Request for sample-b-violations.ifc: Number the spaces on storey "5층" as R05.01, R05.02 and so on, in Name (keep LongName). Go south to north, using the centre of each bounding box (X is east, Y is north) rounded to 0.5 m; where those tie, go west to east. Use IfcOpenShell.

First a look at what the model holds.

```python
import ifcopenshell
import ifcopenshell.util.element
import ifcopenshell.util.placement

model = ifcopenshell.open("sample-b-violations.ifc")
print(model.schema)
storey = next(s for s in model.by_type("IfcBuildingStorey") if s.Name == "5층")
spaces = [e for e in ifcopenshell.util.element.get_decomposition(storey) if e.is_a("IfcSpace")]
for e in sorted(spaces, key=lambda e: e.id()):
    origin = ifcopenshell.util.placement.get_local_placement(e.ObjectPlacement)[:3, 3]
    print(e.id(), e.Name, e.LongName, origin.round(2) + 0.0, sep=" | ")
```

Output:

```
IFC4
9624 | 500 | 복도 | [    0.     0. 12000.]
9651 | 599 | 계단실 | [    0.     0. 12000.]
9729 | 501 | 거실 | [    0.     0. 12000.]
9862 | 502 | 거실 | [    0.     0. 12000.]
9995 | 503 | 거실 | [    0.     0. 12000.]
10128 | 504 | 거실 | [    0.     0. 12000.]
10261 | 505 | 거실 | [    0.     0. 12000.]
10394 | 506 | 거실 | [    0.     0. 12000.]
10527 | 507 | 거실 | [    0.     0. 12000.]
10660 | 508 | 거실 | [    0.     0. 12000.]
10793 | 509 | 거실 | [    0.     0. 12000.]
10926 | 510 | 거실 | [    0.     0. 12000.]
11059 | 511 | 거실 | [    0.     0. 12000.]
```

```python
import ifcopenshell
import ifcopenshell.geom
import ifcopenshell.util.element
import ifcopenshell.util.shape

model = ifcopenshell.open("sample-b-violations.ifc")
settings = ifcopenshell.geom.settings()
settings.set("use-world-coords", True)


def centre(element):
    shape = ifcopenshell.geom.create_shape(settings, element)
    return ifcopenshell.util.shape.get_bbox_centroid(shape.geometry)


storey = next(s for s in model.by_type("IfcBuildingStorey") if s.Name == "5층")
spaces = [e for e in ifcopenshell.util.element.get_decomposition(storey) if e.is_a("IfcSpace")]

# Insertion points can sit at a corner or the storey origin, so sort by the geometry (in metres).
centres = {e: centre(e) for e in spaces}
spaces.sort(key=lambda e: (round(centres[e][1] / 0.5), centres[e][0]))

for i, e in enumerate(spaces, start=1):
    number = f"R05.{i:02d}"
    e.Name = number
    print(e.id(), number)

model.write("sample-b-violations_rev.ifc")
```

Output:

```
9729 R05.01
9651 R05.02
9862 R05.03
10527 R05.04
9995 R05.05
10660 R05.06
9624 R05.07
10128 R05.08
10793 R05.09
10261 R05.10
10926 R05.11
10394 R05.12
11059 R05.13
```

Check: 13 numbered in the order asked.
